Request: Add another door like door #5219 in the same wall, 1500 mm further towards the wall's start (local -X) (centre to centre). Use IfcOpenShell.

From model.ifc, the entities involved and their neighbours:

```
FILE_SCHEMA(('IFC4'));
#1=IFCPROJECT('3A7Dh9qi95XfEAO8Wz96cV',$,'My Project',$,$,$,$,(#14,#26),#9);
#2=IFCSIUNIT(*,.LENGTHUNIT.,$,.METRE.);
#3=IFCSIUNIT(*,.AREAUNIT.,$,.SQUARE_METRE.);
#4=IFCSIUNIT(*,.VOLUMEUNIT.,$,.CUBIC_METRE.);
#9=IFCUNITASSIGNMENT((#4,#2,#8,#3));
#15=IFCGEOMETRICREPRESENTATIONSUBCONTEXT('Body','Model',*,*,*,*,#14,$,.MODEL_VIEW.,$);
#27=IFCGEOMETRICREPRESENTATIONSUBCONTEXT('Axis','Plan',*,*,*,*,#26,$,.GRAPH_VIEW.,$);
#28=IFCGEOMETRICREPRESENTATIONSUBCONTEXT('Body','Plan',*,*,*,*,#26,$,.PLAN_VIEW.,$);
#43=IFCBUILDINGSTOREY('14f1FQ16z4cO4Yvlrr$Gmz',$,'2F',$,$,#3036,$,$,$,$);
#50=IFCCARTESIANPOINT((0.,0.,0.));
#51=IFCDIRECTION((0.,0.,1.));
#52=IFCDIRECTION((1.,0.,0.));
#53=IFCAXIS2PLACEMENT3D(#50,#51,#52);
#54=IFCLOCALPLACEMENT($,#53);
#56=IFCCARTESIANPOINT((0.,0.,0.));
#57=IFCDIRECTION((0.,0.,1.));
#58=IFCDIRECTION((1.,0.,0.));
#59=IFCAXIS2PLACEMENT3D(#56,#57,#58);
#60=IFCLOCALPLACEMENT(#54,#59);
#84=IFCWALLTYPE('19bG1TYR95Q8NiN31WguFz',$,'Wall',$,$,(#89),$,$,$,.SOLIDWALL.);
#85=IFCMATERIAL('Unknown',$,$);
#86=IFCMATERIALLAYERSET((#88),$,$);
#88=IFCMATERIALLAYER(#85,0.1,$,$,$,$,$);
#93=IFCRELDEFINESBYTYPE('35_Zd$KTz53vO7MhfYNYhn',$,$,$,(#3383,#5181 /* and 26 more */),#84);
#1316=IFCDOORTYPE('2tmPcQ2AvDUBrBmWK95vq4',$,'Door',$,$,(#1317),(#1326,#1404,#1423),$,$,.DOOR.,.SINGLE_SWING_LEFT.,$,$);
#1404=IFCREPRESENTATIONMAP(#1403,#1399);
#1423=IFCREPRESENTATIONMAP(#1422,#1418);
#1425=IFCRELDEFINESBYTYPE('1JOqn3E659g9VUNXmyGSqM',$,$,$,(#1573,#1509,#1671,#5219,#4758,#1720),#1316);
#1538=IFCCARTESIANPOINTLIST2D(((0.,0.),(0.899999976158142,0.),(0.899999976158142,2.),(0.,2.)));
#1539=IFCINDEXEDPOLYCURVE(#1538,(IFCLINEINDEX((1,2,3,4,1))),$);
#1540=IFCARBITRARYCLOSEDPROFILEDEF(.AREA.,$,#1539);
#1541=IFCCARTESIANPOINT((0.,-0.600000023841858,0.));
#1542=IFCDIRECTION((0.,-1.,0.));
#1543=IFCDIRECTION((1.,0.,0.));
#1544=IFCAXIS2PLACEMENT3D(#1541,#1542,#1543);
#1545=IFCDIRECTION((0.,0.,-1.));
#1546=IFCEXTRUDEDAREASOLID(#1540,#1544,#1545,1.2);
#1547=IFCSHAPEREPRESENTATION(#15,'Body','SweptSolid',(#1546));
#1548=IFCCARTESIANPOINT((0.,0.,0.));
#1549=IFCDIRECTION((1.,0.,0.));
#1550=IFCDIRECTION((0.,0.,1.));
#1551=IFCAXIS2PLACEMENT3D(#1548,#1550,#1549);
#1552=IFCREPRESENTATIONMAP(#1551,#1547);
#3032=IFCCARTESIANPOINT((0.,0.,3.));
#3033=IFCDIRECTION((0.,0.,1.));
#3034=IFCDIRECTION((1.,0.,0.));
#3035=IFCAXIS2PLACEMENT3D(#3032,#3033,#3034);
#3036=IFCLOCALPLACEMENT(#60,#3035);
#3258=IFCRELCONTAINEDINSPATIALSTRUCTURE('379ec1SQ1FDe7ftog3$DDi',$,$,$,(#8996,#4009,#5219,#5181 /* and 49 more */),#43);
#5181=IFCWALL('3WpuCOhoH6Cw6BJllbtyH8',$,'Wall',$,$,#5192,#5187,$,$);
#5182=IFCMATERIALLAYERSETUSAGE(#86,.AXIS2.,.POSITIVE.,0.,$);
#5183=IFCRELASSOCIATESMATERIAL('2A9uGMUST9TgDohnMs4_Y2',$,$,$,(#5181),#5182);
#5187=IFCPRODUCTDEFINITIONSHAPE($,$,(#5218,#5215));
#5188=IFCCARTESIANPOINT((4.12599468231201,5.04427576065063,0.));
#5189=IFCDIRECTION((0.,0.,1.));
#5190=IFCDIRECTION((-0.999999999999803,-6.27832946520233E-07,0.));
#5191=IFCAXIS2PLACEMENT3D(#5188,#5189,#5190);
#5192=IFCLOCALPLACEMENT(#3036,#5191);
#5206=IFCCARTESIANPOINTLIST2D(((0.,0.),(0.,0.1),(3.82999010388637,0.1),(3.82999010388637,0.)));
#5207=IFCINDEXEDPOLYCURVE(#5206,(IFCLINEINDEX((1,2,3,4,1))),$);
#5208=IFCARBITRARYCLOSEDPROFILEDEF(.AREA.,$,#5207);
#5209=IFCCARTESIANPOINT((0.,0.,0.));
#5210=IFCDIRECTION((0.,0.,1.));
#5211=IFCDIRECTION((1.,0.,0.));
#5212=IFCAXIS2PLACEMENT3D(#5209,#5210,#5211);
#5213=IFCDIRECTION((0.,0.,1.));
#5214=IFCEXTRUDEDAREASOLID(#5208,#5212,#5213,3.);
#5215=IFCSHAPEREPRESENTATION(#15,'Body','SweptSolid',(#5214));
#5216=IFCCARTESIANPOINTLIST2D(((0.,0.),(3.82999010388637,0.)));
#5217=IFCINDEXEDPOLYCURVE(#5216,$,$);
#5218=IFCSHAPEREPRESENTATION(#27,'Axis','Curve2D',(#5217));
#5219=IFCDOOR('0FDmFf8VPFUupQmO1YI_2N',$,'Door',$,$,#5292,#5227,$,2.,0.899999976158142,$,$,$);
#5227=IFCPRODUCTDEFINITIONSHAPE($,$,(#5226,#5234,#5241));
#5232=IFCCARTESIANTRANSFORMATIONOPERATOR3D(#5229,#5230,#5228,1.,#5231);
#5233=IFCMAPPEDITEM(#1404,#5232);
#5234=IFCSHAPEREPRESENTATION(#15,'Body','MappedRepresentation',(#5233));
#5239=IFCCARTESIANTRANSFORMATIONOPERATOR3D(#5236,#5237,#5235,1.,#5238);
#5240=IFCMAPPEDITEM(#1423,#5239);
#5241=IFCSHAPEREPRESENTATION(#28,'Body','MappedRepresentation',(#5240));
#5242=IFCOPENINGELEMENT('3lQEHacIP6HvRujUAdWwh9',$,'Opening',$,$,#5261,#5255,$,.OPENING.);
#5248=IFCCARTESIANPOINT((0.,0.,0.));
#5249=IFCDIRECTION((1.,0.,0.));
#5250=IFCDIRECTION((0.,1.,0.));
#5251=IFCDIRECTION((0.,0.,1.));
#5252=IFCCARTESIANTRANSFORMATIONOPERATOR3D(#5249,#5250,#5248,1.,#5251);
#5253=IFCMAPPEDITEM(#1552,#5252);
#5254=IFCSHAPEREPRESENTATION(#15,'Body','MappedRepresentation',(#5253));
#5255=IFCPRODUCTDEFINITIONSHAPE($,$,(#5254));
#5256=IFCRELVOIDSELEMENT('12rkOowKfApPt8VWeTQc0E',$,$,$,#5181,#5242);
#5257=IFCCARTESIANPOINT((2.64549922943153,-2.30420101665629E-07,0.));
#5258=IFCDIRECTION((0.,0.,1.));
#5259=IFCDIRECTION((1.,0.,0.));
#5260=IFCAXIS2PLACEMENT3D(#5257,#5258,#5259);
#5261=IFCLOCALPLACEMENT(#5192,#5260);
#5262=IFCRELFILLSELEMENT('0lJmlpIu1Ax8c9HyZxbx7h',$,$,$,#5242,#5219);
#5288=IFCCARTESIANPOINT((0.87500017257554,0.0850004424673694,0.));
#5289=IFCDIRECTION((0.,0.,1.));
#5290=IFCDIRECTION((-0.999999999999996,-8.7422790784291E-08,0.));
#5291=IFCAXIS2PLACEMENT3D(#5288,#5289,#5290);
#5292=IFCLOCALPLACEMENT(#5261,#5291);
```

```python
import ifcopenshell
import ifcopenshell.api.feature
import ifcopenshell.api.geometry
import ifcopenshell.api.root
import ifcopenshell.geom
import ifcopenshell.util.element
import ifcopenshell.util.placement
import ifcopenshell.util.shape
import ifcopenshell.util.unit

model = ifcopenshell.open("model.ifc")
unit_scale = ifcopenshell.util.unit.calculate_unit_scale(model)
settings = ifcopenshell.geom.settings()


def volume(element):
    """Net volume in cubic metres, openings subtracted."""
    shape = ifcopenshell.geom.create_shape(settings, element)
    return ifcopenshell.util.shape.get_volume(shape.geometry)


door = model.by_guid("0FDmFf8VPFUupQmO1YI_2N")
opening = door.FillsVoids[0].RelatingOpeningElement
wall = opening.VoidsElements[0].RelatingBuildingElement
before = volume(wall)
shift = ifcopenshell.util.placement.get_local_placement(wall.ObjectPlacement)[:3, 0] * -1.5 / unit_scale

# copy_class copies the void relationship, type, container and properties, but no geometry.
new_opening = ifcopenshell.api.root.copy_class(model, product=opening)
new_opening.Representation = ifcopenshell.util.element.copy_deep(
    model, opening.Representation, exclude=["IfcGeometricRepresentationContext", "IfcRepresentationMap"]
)
new_door = ifcopenshell.api.root.copy_class(model, product=door)
new_door.Representation = ifcopenshell.util.element.copy_deep(
    model, door.Representation, exclude=["IfcGeometricRepresentationContext", "IfcRepresentationMap"]
)
ifcopenshell.api.feature.add_filling(model, opening=new_opening, element=new_door)

for old, new in ((opening, new_opening), (door, new_door)):
    matrix = ifcopenshell.util.placement.get_local_placement(old.ObjectPlacement)
    matrix[:3, 3] += shift
    ifcopenshell.api.geometry.edit_object_placement(model, product=new, matrix=matrix, is_si=False)

after = volume(wall)

print(f"wall volume {before:.3f} -> {after:.3f} m3")

model.write("model_rev.ifc")
```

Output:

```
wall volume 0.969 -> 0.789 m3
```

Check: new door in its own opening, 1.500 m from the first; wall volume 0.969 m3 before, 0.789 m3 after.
